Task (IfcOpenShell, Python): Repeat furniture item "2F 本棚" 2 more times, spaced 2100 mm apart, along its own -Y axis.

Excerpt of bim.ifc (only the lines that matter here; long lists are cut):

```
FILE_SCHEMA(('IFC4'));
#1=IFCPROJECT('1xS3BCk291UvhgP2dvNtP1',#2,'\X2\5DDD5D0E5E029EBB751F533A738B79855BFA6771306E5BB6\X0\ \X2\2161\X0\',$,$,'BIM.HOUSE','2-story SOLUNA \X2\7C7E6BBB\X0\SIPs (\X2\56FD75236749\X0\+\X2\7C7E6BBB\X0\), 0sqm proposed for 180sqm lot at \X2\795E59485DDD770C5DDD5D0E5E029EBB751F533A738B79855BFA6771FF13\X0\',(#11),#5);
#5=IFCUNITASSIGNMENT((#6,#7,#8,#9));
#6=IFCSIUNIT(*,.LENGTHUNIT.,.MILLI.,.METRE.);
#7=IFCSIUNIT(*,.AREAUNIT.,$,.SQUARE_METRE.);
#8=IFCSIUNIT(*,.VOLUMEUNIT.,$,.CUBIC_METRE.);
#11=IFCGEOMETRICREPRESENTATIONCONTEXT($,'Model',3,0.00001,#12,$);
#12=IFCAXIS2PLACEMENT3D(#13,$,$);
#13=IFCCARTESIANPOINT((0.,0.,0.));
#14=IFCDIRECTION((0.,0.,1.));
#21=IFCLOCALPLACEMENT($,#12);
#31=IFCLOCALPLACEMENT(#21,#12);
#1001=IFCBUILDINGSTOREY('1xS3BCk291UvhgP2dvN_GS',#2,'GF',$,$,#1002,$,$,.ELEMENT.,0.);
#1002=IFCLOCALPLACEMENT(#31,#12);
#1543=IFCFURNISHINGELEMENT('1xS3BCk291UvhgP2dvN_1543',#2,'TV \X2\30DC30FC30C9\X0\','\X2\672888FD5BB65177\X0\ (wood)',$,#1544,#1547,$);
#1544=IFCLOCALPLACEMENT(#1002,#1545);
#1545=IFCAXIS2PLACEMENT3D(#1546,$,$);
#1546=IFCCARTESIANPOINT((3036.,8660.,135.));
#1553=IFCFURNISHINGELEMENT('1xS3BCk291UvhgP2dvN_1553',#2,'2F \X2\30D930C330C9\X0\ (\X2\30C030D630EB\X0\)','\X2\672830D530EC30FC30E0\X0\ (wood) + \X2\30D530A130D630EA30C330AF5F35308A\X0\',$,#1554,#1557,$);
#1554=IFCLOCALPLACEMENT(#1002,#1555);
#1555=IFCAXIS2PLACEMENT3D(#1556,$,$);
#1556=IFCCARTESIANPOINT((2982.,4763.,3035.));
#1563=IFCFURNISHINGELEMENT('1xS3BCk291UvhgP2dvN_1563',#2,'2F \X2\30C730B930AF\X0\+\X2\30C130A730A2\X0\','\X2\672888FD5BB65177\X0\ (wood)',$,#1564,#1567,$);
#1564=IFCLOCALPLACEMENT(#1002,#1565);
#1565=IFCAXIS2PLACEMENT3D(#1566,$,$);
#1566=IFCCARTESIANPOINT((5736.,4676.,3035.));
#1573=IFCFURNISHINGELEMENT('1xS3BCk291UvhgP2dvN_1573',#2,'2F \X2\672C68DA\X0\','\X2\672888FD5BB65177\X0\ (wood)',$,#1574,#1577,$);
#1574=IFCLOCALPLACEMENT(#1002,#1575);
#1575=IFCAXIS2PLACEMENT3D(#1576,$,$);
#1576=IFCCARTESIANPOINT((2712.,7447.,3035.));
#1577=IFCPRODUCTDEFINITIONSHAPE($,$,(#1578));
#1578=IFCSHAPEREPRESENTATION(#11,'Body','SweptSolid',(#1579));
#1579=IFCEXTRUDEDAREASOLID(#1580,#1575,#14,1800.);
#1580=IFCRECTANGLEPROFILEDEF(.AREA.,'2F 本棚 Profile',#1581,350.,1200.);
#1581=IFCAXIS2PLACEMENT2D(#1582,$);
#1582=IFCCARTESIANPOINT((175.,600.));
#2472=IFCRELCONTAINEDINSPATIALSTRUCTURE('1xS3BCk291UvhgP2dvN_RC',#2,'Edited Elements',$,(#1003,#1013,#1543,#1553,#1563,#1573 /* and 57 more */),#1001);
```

```python
import ifcopenshell
import ifcopenshell.api.geometry
import ifcopenshell.api.root
import ifcopenshell.util.element
import ifcopenshell.util.placement

model = ifcopenshell.open("bim.ifc")


def reuse_history(source, copy):
    """copy_class also copies each property set's owner history, people and application; keep the originals."""
    for rel in copy.IsDefinedBy:
        if rel.is_a("IfcRelDefinesByProperties") and (history := rel.RelatingPropertyDefinition.OwnerHistory):
            rel.RelatingPropertyDefinition.OwnerHistory = source.OwnerHistory
            ifcopenshell.util.element.remove_deep2(model, history)


source = model.by_id(1573)
base = ifcopenshell.util.placement.get_local_placement(source.ObjectPlacement)
step = -base[:3, 1] * 2100.0

for i in range(1, 3):
    copy = ifcopenshell.api.root.copy_class(model, product=source)
    copy.Representation = ifcopenshell.util.element.copy_deep(
        model, source.Representation, exclude=["IfcGeometricRepresentationContext", "IfcRepresentationMap"]
    )
    reuse_history(source, copy)
    matrix = base.copy()
    matrix[:3, 3] += i * step
    print("added at", matrix[:3, 3].round(3) + 0.0)
    ifcopenshell.api.geometry.edit_object_placement(model, product=copy, matrix=matrix, is_si=False)

model.write("bim_updated.ifc")
```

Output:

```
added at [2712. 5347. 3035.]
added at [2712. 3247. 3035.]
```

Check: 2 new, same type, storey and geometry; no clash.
